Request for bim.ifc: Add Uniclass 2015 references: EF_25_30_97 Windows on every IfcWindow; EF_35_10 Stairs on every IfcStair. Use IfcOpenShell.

First a look at what the model holds.

```python
import ifcopenshell

model = ifcopenshell.open("bim.ifc")
print(model.schema)
print("classifications:", [c.Name for c in model.by_type("IfcClassification")])
for ifc_class in ("IfcDoor", "IfcRoof", "IfcStair", "IfcWall", "IfcWindow"):
    print(ifc_class, len(model.by_type(ifc_class)))
```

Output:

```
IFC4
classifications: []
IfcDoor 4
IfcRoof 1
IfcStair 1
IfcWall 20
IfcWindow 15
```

```python
import ifcopenshell
import ifcopenshell.api.classification

model = ifcopenshell.open("bim.ifc")

system = ifcopenshell.api.classification.add_classification(model, classification="Uniclass 2015")

codes = {
    "IfcWindow": ("EF_25_30_97", "Windows"),
    "IfcStair": ("EF_35_10", "Stairs"),
}
for ifc_class, (code, name) in codes.items():
    products = model.by_type(ifc_class)
    ifcopenshell.api.classification.add_reference(
        model, products=products, classification=system, identification=code, name=name
    )
    print(code, len(products))

model.write("bim-out.ifc")
```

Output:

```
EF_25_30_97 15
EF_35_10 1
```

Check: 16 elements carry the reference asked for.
